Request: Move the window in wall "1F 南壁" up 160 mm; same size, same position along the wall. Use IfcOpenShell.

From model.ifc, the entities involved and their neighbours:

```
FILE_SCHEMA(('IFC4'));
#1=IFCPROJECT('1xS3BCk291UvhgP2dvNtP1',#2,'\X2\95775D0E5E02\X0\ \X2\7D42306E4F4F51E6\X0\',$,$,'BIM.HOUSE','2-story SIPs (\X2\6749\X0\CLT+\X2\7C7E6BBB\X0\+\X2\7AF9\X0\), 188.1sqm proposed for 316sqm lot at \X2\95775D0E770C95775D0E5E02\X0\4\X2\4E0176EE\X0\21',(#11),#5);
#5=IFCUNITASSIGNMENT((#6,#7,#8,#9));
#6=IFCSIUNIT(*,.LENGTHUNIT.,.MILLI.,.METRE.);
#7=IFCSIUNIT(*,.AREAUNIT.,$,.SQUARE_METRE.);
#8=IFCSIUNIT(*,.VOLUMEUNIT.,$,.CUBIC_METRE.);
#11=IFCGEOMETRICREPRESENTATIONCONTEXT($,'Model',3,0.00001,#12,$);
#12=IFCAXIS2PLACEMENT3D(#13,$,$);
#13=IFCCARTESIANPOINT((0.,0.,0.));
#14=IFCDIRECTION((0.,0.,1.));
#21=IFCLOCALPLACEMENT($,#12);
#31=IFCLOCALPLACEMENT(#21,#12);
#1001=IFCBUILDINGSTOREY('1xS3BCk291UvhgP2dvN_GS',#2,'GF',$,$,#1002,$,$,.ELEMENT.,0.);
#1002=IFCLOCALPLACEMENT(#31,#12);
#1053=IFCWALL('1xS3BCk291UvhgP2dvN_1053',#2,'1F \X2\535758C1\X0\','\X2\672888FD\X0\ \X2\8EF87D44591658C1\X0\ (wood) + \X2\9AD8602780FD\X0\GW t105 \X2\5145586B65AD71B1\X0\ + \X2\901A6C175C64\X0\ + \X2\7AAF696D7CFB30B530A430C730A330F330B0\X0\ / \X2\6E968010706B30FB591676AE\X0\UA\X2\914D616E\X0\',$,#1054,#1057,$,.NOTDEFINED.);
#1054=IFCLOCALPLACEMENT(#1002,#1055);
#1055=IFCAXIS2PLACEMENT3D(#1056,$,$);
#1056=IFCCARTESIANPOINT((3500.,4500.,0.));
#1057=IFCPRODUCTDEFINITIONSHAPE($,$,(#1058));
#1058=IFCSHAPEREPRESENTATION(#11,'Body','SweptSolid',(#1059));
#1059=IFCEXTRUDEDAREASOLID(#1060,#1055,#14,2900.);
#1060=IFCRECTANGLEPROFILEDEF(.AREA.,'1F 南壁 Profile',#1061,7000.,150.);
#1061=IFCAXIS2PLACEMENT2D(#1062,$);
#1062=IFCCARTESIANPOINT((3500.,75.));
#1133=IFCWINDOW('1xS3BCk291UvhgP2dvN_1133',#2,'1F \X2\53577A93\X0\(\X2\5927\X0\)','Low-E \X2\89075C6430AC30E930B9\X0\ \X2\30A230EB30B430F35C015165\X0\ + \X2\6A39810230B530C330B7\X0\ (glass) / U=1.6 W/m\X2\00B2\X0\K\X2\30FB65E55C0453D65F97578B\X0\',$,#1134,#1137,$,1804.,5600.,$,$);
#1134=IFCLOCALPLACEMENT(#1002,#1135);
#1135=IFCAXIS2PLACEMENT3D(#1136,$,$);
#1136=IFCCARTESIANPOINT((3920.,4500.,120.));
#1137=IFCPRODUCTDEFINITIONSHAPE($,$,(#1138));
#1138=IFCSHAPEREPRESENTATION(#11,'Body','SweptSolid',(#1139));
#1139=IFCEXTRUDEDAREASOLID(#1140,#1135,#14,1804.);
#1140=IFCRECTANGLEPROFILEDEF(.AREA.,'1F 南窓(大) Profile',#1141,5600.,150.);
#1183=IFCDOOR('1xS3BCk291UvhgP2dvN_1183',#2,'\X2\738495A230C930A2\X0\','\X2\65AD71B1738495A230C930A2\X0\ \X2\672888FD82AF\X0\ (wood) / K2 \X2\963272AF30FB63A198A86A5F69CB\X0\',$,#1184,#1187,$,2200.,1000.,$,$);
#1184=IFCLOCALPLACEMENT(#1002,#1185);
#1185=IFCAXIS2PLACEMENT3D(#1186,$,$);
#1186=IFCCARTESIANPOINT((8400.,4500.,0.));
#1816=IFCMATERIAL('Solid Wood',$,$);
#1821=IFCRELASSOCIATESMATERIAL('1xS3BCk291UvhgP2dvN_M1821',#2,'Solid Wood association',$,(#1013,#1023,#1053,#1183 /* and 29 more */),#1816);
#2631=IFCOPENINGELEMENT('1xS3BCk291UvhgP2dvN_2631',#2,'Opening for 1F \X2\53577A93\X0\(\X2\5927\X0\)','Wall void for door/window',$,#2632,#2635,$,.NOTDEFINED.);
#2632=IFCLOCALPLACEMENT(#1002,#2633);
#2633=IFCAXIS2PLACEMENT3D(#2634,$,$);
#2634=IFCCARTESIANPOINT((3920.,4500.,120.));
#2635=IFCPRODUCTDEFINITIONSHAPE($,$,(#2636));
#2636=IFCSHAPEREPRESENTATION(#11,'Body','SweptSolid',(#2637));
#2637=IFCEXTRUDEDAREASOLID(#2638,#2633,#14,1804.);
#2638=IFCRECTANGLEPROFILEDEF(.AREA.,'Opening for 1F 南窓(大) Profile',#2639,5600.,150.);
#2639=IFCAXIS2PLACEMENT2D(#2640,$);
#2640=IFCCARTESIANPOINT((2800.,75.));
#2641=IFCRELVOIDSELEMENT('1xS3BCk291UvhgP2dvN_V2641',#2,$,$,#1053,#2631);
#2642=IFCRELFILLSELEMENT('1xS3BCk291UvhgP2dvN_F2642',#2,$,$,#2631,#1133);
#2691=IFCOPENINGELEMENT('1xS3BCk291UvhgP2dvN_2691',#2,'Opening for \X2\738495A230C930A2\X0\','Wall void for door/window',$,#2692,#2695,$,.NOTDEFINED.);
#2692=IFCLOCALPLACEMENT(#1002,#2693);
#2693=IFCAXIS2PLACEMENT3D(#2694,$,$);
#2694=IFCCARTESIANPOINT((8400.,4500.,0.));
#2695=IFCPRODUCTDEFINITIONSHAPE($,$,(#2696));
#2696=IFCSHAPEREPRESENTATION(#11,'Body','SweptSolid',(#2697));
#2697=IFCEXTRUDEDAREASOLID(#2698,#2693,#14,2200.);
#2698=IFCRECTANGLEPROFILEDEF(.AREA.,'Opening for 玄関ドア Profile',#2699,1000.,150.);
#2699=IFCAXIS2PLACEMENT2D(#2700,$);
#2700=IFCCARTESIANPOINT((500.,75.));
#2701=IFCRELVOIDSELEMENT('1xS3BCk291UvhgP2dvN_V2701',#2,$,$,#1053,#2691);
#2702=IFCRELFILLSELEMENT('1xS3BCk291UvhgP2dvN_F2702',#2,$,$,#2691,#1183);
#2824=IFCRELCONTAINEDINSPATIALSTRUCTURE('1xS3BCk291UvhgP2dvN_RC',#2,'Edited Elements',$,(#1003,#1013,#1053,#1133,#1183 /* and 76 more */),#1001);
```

```python
import numpy as np
import ifcopenshell
import ifcopenshell.api.geometry
import ifcopenshell.util.placement
import ifcopenshell.util.unit

model = ifcopenshell.open("model.ifc")
unit_scale = ifcopenshell.util.unit.calculate_unit_scale(model)

window = model.by_guid("1xS3BCk291UvhgP2dvN_1133")
opening = window.FillsVoids[0].RelatingOpeningElement
dz = 160.0

shift = np.array([0.0, 0.0, dz])
# The window is not placed relative to its opening, so move both.
for product in (opening, window):
    matrix = ifcopenshell.util.placement.get_local_placement(product.ObjectPlacement)
    matrix[:3, 3] += shift
    ifcopenshell.api.geometry.edit_object_placement(model, product=product, matrix=matrix, is_si=False)

print(f"moved by {dz * unit_scale:+.3f} m")

model.write("model_rev.ifc")
```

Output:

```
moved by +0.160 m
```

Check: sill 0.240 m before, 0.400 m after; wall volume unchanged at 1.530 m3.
